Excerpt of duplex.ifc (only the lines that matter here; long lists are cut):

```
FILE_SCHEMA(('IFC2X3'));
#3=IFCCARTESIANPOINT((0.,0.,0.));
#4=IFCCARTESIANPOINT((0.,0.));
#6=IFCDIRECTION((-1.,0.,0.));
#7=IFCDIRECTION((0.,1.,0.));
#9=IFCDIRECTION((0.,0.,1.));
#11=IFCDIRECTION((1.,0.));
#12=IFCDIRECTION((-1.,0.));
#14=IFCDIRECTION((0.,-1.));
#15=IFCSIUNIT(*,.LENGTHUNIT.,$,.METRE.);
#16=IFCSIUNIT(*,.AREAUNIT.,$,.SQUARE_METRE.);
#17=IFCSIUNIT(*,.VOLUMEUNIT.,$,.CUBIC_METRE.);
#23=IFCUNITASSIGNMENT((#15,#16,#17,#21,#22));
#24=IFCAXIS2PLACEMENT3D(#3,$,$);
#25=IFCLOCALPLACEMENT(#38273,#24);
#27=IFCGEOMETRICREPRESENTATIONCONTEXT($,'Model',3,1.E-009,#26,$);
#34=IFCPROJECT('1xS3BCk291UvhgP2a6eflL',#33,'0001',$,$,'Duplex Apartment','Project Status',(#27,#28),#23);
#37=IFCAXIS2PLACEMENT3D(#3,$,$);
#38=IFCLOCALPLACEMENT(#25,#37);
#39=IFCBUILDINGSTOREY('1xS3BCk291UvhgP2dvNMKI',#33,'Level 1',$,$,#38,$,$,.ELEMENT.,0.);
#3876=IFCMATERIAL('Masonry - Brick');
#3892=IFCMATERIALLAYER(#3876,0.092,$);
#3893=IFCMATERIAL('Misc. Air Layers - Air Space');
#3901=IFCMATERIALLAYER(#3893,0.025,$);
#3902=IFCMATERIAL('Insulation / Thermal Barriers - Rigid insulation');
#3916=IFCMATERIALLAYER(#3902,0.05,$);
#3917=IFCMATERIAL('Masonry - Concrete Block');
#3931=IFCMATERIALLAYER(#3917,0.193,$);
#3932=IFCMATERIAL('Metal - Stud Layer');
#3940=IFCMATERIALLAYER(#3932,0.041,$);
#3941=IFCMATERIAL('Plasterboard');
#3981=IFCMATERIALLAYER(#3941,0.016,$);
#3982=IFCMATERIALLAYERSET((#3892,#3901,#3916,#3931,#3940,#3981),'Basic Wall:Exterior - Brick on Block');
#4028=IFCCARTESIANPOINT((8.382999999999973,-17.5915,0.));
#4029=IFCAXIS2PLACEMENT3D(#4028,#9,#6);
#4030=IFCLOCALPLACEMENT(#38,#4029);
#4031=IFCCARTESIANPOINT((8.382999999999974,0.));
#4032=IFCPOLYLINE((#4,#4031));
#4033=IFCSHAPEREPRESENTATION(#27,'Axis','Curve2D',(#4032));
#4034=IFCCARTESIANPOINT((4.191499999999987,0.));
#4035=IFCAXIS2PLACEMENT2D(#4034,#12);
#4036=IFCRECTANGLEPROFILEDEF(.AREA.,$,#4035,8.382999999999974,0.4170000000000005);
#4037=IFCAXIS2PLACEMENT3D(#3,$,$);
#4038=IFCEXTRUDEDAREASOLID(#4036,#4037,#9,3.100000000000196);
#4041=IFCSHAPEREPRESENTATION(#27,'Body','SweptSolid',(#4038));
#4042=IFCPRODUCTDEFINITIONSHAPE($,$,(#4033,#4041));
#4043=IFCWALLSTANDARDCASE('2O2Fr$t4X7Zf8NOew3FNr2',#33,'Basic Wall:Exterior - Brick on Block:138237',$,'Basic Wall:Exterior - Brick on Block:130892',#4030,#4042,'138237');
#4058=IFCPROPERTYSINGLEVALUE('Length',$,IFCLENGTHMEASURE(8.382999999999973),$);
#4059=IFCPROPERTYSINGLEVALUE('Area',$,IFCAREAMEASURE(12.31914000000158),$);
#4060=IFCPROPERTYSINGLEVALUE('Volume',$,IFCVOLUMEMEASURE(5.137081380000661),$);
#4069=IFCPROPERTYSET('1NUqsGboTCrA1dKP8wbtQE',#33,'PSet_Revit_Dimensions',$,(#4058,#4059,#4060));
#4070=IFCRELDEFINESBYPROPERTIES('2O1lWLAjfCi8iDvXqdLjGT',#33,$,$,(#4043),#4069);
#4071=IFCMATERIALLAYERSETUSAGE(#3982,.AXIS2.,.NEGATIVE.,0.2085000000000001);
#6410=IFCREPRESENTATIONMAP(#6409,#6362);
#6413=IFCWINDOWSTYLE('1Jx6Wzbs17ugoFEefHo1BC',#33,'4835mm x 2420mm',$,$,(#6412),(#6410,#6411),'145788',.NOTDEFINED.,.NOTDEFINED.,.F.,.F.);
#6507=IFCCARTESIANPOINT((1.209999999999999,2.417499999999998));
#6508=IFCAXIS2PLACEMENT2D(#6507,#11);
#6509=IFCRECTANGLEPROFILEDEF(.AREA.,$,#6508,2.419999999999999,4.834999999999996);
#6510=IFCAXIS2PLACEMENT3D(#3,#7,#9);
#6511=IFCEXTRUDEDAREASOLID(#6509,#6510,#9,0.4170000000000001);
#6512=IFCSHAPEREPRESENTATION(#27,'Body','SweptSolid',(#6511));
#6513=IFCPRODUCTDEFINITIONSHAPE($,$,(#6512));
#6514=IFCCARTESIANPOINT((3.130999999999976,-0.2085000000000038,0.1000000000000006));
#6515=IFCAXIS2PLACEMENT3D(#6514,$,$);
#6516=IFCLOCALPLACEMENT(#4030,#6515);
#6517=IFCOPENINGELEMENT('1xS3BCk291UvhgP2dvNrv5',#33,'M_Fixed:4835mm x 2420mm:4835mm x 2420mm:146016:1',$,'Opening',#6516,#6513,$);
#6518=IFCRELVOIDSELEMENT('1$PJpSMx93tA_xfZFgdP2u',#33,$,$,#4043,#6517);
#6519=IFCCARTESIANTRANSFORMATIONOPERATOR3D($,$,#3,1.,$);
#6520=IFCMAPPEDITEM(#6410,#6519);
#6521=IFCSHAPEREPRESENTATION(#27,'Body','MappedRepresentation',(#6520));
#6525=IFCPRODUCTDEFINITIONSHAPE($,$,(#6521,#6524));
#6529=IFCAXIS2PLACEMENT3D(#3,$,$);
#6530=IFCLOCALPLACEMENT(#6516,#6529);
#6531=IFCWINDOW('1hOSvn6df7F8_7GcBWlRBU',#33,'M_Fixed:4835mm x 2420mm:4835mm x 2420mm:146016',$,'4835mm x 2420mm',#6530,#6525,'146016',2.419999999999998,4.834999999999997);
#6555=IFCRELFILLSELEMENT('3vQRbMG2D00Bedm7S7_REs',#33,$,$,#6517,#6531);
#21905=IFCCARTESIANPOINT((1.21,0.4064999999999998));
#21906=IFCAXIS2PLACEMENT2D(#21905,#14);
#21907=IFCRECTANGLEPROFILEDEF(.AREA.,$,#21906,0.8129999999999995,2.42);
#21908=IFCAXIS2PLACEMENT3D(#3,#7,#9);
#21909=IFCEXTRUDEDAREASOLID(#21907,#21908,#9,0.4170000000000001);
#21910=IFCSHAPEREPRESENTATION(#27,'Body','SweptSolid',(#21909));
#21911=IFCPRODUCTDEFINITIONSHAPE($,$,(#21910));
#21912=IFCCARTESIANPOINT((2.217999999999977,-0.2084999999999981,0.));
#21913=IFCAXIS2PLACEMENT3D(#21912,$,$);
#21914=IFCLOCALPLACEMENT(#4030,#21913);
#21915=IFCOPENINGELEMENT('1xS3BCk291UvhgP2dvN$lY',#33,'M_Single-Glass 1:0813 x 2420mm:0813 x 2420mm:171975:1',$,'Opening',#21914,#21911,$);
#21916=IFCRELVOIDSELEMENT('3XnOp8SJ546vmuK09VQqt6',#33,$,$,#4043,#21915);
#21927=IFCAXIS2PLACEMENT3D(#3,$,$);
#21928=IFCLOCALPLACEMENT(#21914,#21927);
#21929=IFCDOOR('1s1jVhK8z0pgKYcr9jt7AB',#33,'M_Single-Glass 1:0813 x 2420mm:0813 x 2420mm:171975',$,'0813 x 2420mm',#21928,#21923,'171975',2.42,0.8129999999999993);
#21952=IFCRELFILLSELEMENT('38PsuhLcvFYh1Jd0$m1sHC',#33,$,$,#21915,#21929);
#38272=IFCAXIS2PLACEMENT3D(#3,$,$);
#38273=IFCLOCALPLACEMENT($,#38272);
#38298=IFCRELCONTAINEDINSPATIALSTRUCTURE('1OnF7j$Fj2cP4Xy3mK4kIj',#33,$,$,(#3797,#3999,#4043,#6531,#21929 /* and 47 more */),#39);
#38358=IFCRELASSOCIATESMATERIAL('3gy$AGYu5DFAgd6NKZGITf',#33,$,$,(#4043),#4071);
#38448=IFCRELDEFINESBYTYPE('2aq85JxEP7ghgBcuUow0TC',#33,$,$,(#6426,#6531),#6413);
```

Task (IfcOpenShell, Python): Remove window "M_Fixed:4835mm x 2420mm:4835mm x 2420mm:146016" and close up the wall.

```python
import ifcopenshell
import ifcopenshell.api.feature
import ifcopenshell.api.pset
import ifcopenshell.api.root
import ifcopenshell.geom
import ifcopenshell.util.element
import ifcopenshell.util.shape
import ifcopenshell.util.unit

model = ifcopenshell.open("duplex.ifc")
area_scale = ifcopenshell.util.unit.calculate_unit_scale(model, "AREAUNIT")
volume_scale = ifcopenshell.util.unit.calculate_unit_scale(model, "VOLUMEUNIT")
settings = ifcopenshell.geom.settings()


def volume(element):
    """Net volume in cubic metres, openings subtracted."""
    shape = ifcopenshell.geom.create_shape(settings, element)
    return ifcopenshell.util.shape.get_volume(shape.geometry)


window = model.by_guid("1hOSvn6df7F8_7GcBWlRBU")
opening = window.FillsVoids[0].RelatingOpeningElement
wall = opening.VoidsElements[0].RelatingBuildingElement
before = volume(wall)

ifcopenshell.api.root.remove_product(model, product=window)
ifcopenshell.api.feature.remove_feature(model, feature=opening)

after = volume(wall)
thickness = 0.417  # wall thickness in metres

# Update the wall's stored quantities.
pset = model.by_id(ifcopenshell.util.element.get_pset(wall, "PSet_Revit_Dimensions", should_inherit=False)["id"])
ifcopenshell.api.pset.edit_pset(model, pset=pset, properties={
    "Area": model.create_entity("IfcAreaMeasure", after / thickness / area_scale),
    "Volume": model.create_entity("IfcVolumeMeasure", after / volume_scale),
})

print(f"wall volume {before:.3f} -> {after:.3f} m3")

model.write("duplex_edited.ifc")
```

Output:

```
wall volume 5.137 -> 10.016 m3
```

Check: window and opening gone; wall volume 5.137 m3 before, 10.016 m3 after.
